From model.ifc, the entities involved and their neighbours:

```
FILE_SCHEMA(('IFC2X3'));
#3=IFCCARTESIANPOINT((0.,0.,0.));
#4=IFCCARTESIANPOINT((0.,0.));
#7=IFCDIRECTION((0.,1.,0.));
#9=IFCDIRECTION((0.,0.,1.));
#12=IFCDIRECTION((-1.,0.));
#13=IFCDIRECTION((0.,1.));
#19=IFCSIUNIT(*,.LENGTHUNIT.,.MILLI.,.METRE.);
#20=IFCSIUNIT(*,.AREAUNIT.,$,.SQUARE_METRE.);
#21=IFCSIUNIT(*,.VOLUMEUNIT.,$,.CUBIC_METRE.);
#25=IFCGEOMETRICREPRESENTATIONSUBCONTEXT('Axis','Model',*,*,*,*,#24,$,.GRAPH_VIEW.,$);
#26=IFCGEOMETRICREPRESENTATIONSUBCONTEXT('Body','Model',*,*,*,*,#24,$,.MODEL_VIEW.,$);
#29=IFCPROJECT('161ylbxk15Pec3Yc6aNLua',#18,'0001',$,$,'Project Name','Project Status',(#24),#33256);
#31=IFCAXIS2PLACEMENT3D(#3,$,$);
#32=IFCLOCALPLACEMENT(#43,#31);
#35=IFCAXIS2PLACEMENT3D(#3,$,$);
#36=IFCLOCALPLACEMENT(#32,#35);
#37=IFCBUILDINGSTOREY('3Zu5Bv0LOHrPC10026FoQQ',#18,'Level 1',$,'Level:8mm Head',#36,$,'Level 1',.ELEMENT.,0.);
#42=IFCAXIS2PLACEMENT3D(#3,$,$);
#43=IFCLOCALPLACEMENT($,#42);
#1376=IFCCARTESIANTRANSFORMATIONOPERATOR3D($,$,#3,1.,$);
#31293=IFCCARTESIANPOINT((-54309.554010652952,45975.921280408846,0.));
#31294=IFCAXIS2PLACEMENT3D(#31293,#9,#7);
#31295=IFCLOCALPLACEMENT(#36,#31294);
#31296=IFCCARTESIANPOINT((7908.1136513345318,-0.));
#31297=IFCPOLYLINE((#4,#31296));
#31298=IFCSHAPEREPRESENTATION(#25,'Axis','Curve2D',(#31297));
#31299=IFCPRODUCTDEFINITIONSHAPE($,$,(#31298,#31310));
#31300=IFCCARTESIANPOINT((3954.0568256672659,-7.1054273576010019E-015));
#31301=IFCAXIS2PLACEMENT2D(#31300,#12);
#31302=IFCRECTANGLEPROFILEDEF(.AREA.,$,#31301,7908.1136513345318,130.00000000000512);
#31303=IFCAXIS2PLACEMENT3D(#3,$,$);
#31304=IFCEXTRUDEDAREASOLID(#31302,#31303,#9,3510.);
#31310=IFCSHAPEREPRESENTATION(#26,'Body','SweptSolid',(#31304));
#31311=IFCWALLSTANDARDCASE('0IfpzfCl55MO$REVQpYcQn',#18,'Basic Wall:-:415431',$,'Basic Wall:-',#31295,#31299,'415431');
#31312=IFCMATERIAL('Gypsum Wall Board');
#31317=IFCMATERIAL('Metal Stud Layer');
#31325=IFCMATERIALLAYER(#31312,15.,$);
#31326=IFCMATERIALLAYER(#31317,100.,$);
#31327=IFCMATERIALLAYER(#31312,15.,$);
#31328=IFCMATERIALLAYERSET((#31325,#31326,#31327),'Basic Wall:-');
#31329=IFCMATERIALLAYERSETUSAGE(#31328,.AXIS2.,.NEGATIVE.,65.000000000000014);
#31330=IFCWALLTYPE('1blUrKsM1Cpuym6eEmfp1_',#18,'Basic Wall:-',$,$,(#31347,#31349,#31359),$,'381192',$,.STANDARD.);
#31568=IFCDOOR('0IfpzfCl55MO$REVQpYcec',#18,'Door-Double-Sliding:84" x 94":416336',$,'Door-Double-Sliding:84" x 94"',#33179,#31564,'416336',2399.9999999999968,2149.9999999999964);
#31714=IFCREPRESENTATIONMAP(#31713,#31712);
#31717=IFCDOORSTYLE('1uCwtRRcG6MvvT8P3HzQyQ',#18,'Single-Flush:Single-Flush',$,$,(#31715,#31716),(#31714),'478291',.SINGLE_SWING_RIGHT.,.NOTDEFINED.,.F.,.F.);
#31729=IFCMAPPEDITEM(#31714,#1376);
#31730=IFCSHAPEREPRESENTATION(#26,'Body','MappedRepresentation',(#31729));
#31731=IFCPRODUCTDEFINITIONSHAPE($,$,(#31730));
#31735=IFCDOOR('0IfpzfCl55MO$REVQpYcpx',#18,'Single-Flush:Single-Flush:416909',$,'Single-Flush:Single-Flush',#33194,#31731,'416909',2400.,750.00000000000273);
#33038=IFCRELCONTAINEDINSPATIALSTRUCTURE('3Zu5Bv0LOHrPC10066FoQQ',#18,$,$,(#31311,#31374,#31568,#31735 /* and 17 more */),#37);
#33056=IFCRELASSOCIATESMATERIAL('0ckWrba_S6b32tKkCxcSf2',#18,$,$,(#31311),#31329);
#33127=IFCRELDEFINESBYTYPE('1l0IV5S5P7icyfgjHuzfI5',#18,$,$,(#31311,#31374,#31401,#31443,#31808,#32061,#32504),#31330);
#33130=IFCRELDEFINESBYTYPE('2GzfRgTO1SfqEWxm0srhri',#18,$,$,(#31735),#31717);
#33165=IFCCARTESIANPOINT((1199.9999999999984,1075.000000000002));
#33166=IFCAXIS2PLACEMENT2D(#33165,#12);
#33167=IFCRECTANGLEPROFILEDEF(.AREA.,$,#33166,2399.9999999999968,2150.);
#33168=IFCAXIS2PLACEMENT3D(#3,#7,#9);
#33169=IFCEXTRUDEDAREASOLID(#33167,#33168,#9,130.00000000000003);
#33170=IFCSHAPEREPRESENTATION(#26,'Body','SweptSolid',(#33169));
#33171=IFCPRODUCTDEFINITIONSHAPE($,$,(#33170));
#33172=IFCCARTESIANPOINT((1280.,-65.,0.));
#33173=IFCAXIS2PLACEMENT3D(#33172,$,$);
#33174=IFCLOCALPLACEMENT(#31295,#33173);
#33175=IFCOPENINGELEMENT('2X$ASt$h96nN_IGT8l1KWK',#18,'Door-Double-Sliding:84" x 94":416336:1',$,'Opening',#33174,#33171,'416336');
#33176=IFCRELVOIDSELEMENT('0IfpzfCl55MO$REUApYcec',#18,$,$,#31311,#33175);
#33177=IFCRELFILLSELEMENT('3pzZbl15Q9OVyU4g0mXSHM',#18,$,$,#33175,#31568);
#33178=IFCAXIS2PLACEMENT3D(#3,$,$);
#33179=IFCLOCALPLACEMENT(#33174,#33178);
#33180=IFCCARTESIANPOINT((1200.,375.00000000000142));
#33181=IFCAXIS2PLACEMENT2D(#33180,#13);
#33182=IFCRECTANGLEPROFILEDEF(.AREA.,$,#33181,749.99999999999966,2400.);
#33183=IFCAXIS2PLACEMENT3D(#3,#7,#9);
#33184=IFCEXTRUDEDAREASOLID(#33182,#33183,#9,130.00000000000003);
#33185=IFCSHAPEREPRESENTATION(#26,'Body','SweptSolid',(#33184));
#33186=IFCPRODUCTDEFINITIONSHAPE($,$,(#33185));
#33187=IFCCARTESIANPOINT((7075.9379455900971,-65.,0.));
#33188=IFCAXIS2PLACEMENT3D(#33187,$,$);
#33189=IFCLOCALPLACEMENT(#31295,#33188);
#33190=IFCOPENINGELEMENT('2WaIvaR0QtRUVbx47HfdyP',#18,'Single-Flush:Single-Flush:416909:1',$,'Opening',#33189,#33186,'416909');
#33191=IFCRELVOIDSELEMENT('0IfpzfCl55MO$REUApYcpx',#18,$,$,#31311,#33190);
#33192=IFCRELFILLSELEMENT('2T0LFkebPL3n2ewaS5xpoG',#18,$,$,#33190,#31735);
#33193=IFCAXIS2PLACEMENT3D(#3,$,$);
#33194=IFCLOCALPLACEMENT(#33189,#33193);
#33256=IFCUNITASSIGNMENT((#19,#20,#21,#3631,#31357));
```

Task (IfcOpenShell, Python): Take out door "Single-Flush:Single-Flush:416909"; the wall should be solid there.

```python
import ifcopenshell
import ifcopenshell.api.feature
import ifcopenshell.api.root
import ifcopenshell.geom
import ifcopenshell.util.shape

model = ifcopenshell.open("model.ifc")
settings = ifcopenshell.geom.settings()


def volume(element):
    """Net volume in cubic metres, openings subtracted."""
    shape = ifcopenshell.geom.create_shape(settings, element)
    return ifcopenshell.util.shape.get_volume(shape.geometry)


door = model.by_id(31735)
opening = door.FillsVoids[0].RelatingOpeningElement
wall = opening.VoidsElements[0].RelatingBuildingElement
before = volume(wall)

ifcopenshell.api.root.remove_product(model, product=door)
ifcopenshell.api.feature.remove_feature(model, feature=opening)

after = volume(wall)

print(f"wall volume {before:.3f} -> {after:.3f} m3")

model.write("model_edited.ifc")
```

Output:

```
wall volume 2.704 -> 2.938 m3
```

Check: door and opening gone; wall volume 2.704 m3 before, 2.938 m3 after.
